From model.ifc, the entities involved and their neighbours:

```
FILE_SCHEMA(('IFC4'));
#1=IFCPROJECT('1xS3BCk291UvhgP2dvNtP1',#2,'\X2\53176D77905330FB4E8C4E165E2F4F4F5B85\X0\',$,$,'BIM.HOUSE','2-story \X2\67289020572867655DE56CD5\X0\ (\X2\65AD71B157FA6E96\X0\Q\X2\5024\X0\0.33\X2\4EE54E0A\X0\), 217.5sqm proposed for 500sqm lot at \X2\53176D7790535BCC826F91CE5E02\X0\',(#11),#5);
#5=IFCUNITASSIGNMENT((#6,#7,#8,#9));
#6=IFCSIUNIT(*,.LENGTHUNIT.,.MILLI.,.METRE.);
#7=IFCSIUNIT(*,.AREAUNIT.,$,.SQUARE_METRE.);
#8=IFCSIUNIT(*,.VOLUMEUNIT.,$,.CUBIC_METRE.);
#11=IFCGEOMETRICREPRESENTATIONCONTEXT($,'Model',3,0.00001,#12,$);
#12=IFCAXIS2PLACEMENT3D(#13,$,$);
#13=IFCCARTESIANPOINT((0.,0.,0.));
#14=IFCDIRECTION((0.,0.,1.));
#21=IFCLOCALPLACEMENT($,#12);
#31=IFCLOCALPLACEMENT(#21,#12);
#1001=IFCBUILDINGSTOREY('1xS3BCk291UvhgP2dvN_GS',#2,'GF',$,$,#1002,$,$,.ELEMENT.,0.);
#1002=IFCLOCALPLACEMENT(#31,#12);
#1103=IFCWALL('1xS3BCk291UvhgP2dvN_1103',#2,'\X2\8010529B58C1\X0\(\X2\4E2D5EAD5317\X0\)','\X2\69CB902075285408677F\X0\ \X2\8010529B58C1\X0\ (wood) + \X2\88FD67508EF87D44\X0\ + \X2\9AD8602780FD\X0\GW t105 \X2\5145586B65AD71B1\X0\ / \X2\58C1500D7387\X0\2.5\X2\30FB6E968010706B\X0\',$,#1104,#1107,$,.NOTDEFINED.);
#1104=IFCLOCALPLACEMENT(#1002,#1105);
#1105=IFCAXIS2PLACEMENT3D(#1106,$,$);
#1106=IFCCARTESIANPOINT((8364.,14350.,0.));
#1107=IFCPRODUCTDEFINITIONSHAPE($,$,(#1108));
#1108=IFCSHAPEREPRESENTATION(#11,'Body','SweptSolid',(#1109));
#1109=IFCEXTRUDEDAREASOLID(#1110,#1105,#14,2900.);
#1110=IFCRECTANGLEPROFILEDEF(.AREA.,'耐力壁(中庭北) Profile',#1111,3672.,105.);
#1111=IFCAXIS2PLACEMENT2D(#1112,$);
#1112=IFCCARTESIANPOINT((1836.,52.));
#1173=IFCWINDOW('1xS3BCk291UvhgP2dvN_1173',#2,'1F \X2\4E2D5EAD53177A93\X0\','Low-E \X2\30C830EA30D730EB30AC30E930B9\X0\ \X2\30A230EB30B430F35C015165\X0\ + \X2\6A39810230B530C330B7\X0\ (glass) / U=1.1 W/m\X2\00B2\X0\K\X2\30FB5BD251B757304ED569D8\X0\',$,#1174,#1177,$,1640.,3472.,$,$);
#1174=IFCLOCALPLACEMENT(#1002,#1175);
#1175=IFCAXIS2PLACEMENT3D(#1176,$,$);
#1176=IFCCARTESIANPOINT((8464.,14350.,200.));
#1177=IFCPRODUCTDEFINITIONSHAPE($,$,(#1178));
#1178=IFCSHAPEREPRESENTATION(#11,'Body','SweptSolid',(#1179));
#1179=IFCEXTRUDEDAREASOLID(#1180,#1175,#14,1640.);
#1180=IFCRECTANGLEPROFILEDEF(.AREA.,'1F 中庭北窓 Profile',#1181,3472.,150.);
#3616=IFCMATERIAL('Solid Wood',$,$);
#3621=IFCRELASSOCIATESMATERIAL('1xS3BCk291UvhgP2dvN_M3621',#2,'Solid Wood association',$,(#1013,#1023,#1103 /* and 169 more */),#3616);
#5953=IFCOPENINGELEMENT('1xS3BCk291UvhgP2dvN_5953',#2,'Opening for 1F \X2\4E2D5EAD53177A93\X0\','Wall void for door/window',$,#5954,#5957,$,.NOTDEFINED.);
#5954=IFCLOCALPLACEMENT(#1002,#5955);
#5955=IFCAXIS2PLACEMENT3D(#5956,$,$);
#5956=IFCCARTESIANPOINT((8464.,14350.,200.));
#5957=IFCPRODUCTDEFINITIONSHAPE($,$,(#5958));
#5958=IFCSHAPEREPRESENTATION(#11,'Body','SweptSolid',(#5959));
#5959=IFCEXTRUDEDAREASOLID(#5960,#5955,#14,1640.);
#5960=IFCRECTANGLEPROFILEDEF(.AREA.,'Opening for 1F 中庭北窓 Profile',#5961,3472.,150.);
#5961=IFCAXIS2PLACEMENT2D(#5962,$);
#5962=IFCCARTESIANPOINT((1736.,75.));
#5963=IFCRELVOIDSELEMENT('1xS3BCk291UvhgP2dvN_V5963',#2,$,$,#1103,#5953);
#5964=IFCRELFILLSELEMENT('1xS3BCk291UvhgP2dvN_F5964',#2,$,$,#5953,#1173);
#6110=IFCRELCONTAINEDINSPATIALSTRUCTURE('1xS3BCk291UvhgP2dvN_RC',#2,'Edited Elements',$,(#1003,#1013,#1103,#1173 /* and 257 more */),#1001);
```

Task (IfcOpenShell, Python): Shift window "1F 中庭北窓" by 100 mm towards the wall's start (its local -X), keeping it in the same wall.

```python
import ifcopenshell
import ifcopenshell.api.geometry
import ifcopenshell.util.placement
import ifcopenshell.util.unit

model = ifcopenshell.open("model.ifc")
unit_scale = ifcopenshell.util.unit.calculate_unit_scale(model)

window = model.by_id(1173)
opening = window.FillsVoids[0].RelatingOpeningElement
wall = opening.VoidsElements[0].RelatingBuildingElement

wall_matrix = ifcopenshell.util.placement.get_local_placement(wall.ObjectPlacement)
shift = wall_matrix[:3, 0] * -0.1 / unit_scale
before = ifcopenshell.util.placement.get_local_placement(window.ObjectPlacement)[:3, 3].copy()

# The window is not placed relative to its opening, so move both.
for product in (opening, window):
    matrix = ifcopenshell.util.placement.get_local_placement(product.ObjectPlacement)
    matrix[:3, 3] += shift
    ifcopenshell.api.geometry.edit_object_placement(model, product=product, matrix=matrix, is_si=False)

after = ifcopenshell.util.placement.get_local_placement(window.ObjectPlacement)[:3, 3]
print("window moved by", (after - before).round(3) + 0.0)

model.write("model_edited.ifc")
```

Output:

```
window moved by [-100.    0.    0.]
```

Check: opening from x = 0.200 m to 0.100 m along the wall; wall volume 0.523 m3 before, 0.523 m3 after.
